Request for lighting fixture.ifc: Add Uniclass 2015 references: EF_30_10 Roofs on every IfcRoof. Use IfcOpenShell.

First a look at what the model holds.

```python
import ifcopenshell

model = ifcopenshell.open("lighting fixture.ifc")
print(model.schema)
print("classifications:", [c.Name for c in model.by_type("IfcClassification")])
for ifc_class in ("IfcDoor", "IfcRoof", "IfcStair", "IfcWall", "IfcWindow"):
    print(ifc_class, len(model.by_type(ifc_class)))
```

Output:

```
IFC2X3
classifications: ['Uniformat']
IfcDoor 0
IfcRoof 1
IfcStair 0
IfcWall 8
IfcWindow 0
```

```python
import ifcopenshell
import ifcopenshell.api.classification

model = ifcopenshell.open("lighting fixture.ifc")

# IFC2X3 requires Source and Edition and has no link from the project to the system.
system = model.create_entity("IfcClassification", Source="NBS", Edition="2015", Name="Uniclass 2015")

codes = {
    "IfcRoof": ("EF_30_10", "Roofs"),
}
for ifc_class, (code, name) in codes.items():
    products = model.by_type(ifc_class)
    ifcopenshell.api.classification.add_reference(
        model, products=products, classification=system, identification=code, name=name
    )
    print(code, len(products))

model.write("lighting fixture_updated.ifc")
```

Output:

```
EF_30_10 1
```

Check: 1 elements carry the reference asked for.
